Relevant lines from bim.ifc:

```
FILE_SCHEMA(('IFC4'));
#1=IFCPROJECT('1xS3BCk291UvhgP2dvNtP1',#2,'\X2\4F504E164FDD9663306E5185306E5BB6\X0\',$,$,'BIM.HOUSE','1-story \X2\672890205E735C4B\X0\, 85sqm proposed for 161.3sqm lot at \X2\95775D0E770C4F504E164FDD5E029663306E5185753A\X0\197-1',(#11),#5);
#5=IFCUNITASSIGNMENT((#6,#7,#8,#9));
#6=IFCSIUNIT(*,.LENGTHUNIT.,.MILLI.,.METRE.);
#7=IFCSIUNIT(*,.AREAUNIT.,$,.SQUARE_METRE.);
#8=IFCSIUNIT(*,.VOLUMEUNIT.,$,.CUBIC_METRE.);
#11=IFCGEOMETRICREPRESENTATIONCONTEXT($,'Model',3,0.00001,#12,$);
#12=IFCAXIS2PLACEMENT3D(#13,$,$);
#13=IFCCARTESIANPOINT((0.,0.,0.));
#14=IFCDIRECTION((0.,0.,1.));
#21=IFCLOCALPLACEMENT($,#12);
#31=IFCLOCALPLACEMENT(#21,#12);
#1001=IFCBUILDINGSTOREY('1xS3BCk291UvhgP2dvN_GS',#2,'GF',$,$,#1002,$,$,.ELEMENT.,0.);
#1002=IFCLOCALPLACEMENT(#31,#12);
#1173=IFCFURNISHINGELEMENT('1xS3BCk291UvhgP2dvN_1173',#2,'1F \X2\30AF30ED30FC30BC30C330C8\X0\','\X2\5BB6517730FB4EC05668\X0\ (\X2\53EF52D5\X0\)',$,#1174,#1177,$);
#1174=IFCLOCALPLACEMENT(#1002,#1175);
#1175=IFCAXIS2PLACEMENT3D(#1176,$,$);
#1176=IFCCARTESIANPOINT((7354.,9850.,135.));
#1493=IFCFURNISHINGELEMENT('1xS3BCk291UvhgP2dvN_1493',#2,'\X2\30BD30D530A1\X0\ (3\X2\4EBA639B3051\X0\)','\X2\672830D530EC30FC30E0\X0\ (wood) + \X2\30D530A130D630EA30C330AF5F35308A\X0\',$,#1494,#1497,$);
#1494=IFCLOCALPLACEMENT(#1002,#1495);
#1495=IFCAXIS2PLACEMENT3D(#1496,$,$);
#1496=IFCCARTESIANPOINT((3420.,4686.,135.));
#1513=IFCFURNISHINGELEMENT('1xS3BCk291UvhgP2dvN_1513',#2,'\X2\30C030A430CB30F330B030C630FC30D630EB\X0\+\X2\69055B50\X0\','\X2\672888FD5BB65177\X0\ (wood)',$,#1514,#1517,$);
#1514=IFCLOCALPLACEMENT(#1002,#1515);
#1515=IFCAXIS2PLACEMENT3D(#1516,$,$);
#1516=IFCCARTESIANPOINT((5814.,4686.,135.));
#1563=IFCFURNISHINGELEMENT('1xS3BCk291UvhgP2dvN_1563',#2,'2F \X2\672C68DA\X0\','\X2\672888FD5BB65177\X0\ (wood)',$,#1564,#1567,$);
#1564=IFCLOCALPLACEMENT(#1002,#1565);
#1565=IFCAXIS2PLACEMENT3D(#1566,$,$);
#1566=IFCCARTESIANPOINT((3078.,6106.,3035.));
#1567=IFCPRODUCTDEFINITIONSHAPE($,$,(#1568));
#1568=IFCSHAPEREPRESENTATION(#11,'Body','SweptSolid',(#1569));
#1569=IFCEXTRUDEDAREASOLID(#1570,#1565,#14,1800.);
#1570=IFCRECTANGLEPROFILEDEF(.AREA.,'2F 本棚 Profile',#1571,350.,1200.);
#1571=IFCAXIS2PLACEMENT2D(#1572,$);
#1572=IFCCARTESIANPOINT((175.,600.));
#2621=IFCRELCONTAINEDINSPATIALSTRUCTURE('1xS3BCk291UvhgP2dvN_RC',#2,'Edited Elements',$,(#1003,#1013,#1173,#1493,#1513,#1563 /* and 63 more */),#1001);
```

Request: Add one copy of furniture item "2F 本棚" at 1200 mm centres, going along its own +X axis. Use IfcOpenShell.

```python
import ifcopenshell
import ifcopenshell.api.geometry
import ifcopenshell.api.root
import ifcopenshell.util.element
import ifcopenshell.util.placement
import ifcopenshell.util.unit

model = ifcopenshell.open("bim.ifc")
unit_scale = ifcopenshell.util.unit.calculate_unit_scale(model)


def reuse_history(source, copy):
    """copy_class also copies each property set's owner history, people and application; keep the originals."""
    for rel in copy.IsDefinedBy:
        if rel.is_a("IfcRelDefinesByProperties") and (history := rel.RelatingPropertyDefinition.OwnerHistory):
            rel.RelatingPropertyDefinition.OwnerHistory = source.OwnerHistory
            ifcopenshell.util.element.remove_deep2(model, history)


source = model.by_guid("1xS3BCk291UvhgP2dvN_1563")
base = ifcopenshell.util.placement.get_local_placement(source.ObjectPlacement)
step = base[:3, 0] * 1.2 / unit_scale

for i in range(1, 2):
    copy = ifcopenshell.api.root.copy_class(model, product=source)
    copy.Representation = ifcopenshell.util.element.copy_deep(
        model, source.Representation, exclude=["IfcGeometricRepresentationContext", "IfcRepresentationMap"]
    )
    reuse_history(source, copy)
    matrix = base.copy()
    matrix[:3, 3] += i * step
    print("added at", matrix[:3, 3].round(3) + 0.0)
    ifcopenshell.api.geometry.edit_object_placement(model, product=copy, matrix=matrix, is_si=False)

model.write("bim_rev.ifc")
```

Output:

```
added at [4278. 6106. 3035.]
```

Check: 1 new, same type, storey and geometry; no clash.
